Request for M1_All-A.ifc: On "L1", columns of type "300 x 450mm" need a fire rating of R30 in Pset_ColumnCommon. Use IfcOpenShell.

First a look at what the model holds.

```python
import ifcopenshell
import ifcopenshell.util.element

model = ifcopenshell.open("M1_All-A.ifc")
print(model.schema)
storey = next(s for s in model.by_type("IfcBuildingStorey") if s.Name == "L1")
columns = [e for e in ifcopenshell.util.element.get_decomposition(storey) if e.is_a("IfcColumn")]
seen = {}
for e in columns:
    element_type = ifcopenshell.util.element.get_type(e)
    key = (element_type.Name if element_type != e and element_type else None, ifcopenshell.util.element.get_pset(e, "Pset_ColumnCommon", "FireRating"))
    seen[key] = seen.get(key, 0) + 1
for (name, value), count in sorted(seen.items(), key=str):
    print(count, "x", name, "|", value)
```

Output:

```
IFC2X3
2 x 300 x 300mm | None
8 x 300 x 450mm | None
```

```python
import ifcopenshell
import ifcopenshell.api.pset
import ifcopenshell.util.element

model = ifcopenshell.open("M1_All-A.ifc")

storey = next(s for s in model.by_type("IfcBuildingStorey") if s.Name == "L1")
columns = [e for e in ifcopenshell.util.element.get_decomposition(storey) if e.is_a("IfcColumn")]

count = 0
for e in columns:
    element_type = ifcopenshell.util.element.get_type(e)
    if element_type in (None, e) or element_type.Name != "300 x 450mm":
        continue
    # add_pset returns the element's existing set when there is one.
    pset = ifcopenshell.api.pset.add_pset(model, product=e, name="Pset_ColumnCommon")
    ifcopenshell.api.pset.edit_pset(model, pset=pset, properties={"FireRating": "R30"})
    count += 1

print(count, "columns updated")

model.write("M1_All-A_v2.ifc")
```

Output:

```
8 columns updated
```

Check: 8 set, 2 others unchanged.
